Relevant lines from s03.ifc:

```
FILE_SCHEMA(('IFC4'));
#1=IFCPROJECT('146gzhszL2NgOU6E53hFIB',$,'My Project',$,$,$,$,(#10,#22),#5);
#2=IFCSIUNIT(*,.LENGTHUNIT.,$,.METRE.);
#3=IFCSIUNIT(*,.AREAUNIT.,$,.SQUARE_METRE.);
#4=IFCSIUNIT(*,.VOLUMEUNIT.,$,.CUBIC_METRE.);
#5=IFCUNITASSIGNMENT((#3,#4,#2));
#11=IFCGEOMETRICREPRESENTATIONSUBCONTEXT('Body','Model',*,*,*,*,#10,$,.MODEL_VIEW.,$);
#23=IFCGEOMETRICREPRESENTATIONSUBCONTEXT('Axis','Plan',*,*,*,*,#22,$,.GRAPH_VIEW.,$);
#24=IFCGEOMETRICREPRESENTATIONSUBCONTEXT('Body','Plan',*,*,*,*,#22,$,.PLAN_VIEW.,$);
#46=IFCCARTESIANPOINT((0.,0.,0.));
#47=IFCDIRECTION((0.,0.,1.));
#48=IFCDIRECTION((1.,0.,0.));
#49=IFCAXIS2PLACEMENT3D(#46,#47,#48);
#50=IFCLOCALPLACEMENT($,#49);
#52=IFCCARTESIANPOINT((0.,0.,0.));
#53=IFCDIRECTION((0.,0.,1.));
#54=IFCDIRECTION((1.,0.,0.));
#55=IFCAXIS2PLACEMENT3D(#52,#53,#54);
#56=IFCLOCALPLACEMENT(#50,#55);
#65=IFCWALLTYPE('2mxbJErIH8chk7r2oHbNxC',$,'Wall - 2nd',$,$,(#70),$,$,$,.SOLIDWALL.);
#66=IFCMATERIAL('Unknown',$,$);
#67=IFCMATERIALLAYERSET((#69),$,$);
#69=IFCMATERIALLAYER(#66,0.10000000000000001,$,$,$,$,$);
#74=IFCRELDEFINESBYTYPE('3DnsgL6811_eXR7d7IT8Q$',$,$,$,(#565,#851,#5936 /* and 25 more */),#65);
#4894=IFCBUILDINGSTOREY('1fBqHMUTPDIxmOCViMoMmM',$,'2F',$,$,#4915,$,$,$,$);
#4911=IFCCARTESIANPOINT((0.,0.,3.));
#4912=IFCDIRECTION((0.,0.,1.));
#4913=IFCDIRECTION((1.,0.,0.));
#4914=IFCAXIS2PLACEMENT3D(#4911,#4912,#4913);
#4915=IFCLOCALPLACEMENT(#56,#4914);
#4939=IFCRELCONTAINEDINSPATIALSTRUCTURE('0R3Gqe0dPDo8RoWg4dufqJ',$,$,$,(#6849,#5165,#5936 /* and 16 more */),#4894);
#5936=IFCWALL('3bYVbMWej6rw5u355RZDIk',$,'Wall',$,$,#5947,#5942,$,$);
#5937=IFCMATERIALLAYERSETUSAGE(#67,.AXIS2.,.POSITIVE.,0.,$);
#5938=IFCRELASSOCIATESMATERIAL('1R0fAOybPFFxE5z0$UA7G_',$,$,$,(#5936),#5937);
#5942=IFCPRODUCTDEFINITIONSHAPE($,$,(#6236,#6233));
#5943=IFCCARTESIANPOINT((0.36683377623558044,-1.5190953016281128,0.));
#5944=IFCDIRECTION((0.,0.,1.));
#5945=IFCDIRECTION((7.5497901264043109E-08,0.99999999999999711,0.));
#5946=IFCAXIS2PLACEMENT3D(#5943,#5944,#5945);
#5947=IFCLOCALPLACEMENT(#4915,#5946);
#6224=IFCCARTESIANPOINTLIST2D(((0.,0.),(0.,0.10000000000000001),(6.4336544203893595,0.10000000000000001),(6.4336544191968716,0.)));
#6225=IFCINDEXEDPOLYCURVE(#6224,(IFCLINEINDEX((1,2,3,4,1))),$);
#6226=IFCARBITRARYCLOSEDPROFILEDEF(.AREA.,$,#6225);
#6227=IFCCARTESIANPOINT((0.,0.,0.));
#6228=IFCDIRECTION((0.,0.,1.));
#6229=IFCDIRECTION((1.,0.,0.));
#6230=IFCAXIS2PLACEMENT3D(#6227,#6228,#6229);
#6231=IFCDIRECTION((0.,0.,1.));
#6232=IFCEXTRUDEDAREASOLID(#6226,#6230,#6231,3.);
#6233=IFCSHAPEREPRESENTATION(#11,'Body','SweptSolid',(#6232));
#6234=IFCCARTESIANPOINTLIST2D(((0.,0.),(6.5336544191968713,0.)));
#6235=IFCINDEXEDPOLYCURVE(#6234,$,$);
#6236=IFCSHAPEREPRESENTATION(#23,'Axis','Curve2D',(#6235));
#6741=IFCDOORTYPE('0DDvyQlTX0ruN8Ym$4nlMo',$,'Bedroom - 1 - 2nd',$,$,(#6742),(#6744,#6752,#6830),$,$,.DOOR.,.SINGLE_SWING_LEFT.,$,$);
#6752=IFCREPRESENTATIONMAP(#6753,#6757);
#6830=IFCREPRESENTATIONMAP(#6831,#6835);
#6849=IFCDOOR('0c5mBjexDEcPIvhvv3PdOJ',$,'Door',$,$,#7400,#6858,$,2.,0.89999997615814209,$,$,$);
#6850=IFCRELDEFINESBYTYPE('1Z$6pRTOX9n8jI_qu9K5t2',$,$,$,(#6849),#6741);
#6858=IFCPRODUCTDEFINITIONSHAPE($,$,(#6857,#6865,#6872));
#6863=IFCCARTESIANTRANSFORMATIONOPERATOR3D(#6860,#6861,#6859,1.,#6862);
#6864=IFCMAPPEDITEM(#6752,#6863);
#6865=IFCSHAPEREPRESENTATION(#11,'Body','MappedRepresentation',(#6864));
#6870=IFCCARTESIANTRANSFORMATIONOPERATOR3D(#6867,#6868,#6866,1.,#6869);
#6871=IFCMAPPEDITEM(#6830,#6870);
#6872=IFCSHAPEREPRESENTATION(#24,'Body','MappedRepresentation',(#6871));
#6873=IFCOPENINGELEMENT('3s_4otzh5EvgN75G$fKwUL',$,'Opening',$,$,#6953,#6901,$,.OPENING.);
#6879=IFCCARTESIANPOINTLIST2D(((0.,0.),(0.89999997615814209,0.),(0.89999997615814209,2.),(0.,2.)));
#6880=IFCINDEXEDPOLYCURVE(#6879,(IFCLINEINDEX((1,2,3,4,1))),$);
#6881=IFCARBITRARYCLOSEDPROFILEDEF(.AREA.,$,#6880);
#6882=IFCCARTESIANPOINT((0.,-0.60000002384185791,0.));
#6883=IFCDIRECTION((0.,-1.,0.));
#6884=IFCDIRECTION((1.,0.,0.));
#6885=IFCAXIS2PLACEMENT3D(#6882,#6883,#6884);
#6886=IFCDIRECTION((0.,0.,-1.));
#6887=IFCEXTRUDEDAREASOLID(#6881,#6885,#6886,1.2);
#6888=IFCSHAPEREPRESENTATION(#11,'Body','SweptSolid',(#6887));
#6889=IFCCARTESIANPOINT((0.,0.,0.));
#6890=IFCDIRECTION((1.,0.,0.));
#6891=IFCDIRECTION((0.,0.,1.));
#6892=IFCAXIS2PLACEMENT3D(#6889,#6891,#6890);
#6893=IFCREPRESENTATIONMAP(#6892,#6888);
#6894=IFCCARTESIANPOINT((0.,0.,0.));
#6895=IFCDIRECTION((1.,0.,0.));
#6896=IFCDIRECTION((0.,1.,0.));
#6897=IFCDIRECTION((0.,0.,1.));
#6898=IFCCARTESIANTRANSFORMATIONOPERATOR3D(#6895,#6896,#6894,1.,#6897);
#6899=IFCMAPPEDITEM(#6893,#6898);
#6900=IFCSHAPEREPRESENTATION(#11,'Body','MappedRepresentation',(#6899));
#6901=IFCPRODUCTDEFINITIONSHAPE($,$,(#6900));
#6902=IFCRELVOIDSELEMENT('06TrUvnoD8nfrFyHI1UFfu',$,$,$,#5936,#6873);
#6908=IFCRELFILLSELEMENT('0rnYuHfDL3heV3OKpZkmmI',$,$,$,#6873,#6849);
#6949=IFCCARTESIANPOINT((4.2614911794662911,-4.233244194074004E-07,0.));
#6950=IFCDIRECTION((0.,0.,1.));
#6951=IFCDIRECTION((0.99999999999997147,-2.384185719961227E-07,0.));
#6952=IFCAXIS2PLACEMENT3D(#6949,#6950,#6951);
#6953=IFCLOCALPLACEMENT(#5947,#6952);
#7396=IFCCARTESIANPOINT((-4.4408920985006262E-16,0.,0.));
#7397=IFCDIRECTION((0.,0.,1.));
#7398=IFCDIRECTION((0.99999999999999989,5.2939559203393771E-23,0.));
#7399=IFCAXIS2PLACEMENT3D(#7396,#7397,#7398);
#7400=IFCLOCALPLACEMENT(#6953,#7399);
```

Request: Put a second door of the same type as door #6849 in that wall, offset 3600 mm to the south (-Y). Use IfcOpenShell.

```python
import ifcopenshell
import ifcopenshell.api.feature
import ifcopenshell.api.geometry
import ifcopenshell.api.root
import ifcopenshell.geom
import ifcopenshell.util.element
import ifcopenshell.util.placement
import ifcopenshell.util.shape
import ifcopenshell.util.unit

model = ifcopenshell.open("s03.ifc")
unit_scale = ifcopenshell.util.unit.calculate_unit_scale(model)
settings = ifcopenshell.geom.settings()


def volume(element):
    """Net volume in cubic metres, openings subtracted."""
    shape = ifcopenshell.geom.create_shape(settings, element)
    return ifcopenshell.util.shape.get_volume(shape.geometry)


door = model.by_guid("0c5mBjexDEcPIvhvv3PdOJ")
opening = door.FillsVoids[0].RelatingOpeningElement
wall = opening.VoidsElements[0].RelatingBuildingElement
before = volume(wall)
shift = ifcopenshell.util.placement.get_local_placement(wall.ObjectPlacement)[:3, 0] * -3.6 / unit_scale

# copy_class copies the void relationship, type, container and properties, but no geometry.
new_opening = ifcopenshell.api.root.copy_class(model, product=opening)
new_opening.Representation = ifcopenshell.util.element.copy_deep(
    model, opening.Representation, exclude=["IfcGeometricRepresentationContext", "IfcRepresentationMap"]
)
new_door = ifcopenshell.api.root.copy_class(model, product=door)
new_door.Representation = ifcopenshell.util.element.copy_deep(
    model, door.Representation, exclude=["IfcGeometricRepresentationContext", "IfcRepresentationMap"]
)
ifcopenshell.api.feature.add_filling(model, opening=new_opening, element=new_door)

for old, new in ((opening, new_opening), (door, new_door)):
    matrix = ifcopenshell.util.placement.get_local_placement(old.ObjectPlacement)
    matrix[:3, 3] += shift
    ifcopenshell.api.geometry.edit_object_placement(model, product=new, matrix=matrix, is_si=False)

after = volume(wall)

print(f"wall volume {before:.3f} -> {after:.3f} m3")

model.write("s03_updated.ifc")
```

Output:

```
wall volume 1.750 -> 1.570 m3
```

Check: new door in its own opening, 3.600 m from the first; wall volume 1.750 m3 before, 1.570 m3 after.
